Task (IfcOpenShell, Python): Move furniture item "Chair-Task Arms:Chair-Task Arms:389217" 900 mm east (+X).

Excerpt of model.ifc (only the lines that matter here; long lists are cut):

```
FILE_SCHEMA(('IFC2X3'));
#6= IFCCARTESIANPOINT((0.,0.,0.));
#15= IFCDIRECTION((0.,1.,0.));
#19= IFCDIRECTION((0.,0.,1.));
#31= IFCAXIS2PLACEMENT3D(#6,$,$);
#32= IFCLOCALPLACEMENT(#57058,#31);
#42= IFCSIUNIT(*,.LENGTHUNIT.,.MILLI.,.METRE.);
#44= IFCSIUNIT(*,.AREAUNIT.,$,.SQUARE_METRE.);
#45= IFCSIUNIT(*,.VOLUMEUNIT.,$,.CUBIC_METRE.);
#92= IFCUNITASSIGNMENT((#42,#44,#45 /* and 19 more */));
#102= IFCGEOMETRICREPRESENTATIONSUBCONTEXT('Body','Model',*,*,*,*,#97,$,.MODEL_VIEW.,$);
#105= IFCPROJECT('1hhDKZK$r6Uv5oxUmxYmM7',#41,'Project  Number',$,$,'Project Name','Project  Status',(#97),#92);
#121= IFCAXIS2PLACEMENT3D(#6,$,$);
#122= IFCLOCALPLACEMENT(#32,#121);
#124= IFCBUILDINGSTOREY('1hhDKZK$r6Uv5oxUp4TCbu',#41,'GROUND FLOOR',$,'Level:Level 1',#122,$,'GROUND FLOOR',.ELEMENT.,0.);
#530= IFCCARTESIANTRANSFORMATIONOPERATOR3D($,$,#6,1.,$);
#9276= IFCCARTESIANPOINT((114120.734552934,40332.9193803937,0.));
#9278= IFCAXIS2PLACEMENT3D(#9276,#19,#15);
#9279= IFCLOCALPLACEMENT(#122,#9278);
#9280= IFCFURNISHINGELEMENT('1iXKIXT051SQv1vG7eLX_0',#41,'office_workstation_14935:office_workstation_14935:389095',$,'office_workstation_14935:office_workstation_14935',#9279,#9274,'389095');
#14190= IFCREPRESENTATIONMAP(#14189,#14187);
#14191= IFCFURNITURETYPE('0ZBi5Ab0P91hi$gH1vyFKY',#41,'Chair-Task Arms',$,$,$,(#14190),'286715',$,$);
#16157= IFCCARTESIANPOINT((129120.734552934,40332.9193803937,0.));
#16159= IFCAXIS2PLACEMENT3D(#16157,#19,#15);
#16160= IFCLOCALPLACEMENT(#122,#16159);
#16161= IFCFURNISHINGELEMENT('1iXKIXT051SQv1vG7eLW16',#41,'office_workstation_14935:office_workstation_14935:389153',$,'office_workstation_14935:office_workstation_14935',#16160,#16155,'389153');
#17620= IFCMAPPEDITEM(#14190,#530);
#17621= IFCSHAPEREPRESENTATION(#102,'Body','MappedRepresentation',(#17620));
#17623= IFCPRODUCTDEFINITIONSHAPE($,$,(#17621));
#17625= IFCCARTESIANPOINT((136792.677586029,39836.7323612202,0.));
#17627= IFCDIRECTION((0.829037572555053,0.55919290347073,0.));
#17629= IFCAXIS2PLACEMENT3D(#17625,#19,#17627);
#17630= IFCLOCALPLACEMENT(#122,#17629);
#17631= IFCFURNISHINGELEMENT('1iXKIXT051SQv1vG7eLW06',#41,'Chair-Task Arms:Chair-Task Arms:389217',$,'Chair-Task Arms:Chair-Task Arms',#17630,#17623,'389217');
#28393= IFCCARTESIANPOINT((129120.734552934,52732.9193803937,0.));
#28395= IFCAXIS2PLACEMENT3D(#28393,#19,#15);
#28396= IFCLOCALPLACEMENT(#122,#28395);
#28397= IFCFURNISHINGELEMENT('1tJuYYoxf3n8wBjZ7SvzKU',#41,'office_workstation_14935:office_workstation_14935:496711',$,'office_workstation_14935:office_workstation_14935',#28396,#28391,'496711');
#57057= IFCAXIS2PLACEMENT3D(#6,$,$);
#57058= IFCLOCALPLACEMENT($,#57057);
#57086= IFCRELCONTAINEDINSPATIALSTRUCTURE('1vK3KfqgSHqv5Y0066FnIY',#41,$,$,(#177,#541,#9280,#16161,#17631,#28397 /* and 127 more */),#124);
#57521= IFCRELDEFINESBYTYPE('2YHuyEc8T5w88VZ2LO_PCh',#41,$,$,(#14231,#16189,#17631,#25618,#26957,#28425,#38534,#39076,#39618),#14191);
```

```python
import ifcopenshell
import ifcopenshell.api.geometry
import ifcopenshell.util.placement

model = ifcopenshell.open("model.ifc")

item = model.by_guid("1iXKIXT051SQv1vG7eLW06")
matrix = ifcopenshell.util.placement.get_local_placement(item.ObjectPlacement)
matrix[0, 3] += 900.0
ifcopenshell.api.geometry.edit_object_placement(model, product=item, matrix=matrix, is_si=False)

print(ifcopenshell.util.placement.get_local_placement(item.ObjectPlacement).round(3) + 0.0)

model.write("model_v2.ifc")
```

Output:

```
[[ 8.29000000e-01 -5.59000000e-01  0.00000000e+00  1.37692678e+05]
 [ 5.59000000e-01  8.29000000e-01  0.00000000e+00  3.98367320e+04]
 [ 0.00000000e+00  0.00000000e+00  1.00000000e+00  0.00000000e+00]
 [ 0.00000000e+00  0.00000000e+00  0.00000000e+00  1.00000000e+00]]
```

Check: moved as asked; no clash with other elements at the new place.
